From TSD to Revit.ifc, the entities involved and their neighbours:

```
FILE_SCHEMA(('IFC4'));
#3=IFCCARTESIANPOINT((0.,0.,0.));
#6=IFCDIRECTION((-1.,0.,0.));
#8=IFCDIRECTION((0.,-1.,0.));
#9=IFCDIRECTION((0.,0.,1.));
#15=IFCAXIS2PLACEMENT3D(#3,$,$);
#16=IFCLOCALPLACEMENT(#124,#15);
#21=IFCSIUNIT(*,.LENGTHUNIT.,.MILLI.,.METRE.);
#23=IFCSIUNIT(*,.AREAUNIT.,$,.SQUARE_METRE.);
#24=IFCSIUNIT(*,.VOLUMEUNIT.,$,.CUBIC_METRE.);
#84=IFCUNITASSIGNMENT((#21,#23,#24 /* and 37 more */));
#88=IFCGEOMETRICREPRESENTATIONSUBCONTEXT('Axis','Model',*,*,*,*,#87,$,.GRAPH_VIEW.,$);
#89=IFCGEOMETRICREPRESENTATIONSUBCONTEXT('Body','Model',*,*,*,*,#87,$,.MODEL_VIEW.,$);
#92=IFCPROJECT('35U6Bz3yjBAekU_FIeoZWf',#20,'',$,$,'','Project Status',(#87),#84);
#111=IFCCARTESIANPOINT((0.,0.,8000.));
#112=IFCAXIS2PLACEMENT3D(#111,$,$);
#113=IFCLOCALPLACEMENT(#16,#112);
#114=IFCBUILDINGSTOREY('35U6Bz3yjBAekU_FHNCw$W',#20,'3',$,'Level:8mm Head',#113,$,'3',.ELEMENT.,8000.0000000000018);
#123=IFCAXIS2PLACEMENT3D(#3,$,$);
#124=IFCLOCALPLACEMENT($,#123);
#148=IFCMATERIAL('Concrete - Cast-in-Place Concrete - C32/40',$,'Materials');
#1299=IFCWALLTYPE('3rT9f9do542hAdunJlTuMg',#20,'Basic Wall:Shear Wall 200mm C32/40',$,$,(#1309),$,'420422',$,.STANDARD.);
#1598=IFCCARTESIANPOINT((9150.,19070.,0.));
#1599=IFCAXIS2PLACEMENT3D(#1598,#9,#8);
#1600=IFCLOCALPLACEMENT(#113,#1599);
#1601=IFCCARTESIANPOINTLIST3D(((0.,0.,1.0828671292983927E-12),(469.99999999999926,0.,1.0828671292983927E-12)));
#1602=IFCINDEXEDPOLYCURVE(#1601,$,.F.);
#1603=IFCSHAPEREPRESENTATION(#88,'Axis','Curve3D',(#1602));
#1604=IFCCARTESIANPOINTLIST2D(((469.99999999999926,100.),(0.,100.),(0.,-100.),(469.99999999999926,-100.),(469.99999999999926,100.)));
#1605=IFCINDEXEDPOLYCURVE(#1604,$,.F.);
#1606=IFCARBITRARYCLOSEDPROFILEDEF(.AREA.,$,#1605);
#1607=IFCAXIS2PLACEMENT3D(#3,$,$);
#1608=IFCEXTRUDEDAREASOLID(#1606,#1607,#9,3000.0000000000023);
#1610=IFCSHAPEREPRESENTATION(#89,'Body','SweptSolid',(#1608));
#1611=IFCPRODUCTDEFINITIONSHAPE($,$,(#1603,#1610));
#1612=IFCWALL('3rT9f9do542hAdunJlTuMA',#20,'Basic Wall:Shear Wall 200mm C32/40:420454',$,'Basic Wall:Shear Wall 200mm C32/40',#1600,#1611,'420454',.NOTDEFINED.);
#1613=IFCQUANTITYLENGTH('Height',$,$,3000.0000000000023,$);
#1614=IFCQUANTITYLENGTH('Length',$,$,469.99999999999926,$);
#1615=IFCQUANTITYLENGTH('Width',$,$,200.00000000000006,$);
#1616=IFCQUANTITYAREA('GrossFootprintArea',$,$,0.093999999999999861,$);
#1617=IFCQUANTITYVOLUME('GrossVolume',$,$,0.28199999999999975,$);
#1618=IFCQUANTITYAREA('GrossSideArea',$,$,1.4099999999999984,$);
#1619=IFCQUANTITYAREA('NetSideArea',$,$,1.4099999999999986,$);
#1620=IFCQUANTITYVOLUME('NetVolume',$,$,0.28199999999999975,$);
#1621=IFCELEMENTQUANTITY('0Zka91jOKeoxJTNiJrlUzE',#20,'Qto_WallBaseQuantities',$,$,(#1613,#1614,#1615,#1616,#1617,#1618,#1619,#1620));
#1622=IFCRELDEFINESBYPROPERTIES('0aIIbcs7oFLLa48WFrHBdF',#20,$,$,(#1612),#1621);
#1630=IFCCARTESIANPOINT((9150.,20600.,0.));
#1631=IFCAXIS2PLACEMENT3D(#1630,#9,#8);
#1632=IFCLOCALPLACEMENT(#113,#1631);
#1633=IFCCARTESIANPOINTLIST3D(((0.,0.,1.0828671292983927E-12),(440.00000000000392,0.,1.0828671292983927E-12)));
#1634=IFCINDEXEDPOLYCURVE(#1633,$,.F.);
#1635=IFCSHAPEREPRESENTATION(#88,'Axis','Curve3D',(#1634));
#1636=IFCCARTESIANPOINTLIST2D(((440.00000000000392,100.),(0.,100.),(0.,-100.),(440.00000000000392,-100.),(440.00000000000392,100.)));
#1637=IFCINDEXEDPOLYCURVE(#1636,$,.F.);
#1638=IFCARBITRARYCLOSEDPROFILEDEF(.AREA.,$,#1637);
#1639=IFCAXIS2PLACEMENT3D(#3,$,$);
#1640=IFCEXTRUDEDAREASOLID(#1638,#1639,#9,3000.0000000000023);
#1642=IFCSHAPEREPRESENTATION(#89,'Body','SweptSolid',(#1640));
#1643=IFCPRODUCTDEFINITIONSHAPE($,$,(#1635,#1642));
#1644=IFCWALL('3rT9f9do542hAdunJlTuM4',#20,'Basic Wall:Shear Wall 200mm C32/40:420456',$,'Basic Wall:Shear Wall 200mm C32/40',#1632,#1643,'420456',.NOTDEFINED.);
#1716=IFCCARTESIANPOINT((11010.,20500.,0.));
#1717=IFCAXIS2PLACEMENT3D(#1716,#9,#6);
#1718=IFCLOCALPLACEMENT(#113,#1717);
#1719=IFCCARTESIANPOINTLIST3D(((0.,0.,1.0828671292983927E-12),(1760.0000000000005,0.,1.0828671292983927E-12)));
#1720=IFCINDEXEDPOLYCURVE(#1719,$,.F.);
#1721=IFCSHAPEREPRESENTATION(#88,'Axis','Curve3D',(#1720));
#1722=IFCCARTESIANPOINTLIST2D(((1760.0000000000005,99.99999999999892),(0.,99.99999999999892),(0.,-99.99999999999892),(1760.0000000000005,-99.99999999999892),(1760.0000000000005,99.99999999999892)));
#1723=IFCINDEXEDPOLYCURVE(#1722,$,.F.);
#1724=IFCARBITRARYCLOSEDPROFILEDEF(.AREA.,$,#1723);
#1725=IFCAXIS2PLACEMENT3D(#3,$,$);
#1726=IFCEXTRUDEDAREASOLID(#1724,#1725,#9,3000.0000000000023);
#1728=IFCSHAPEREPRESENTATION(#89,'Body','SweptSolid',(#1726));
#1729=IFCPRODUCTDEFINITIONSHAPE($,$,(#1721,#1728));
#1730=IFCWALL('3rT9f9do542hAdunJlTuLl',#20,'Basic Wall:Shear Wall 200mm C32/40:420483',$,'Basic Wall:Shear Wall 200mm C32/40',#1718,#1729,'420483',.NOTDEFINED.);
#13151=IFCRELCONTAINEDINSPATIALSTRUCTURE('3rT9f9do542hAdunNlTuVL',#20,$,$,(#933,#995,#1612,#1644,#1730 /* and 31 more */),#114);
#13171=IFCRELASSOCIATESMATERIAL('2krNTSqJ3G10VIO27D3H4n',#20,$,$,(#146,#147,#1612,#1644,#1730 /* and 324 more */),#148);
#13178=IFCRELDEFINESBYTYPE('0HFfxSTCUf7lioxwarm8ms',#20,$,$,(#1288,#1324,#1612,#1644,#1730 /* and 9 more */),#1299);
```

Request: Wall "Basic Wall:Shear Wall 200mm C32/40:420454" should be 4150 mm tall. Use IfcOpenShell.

```python
import ifcopenshell
import ifcopenshell.api.pset
import ifcopenshell.geom
import ifcopenshell.util.element
import ifcopenshell.util.representation
import ifcopenshell.util.shape
import ifcopenshell.util.unit

model = ifcopenshell.open("TSD to Revit.ifc")
unit_scale = ifcopenshell.util.unit.calculate_unit_scale(model)
area_scale = ifcopenshell.util.unit.calculate_unit_scale(model, "AREAUNIT")
volume_scale = ifcopenshell.util.unit.calculate_unit_scale(model, "VOLUMEUNIT")
settings = ifcopenshell.geom.settings()


def volume(element):
    """Net volume in cubic metres, openings subtracted."""
    shape = ifcopenshell.geom.create_shape(settings, element)
    return ifcopenshell.util.shape.get_volume(shape.geometry)


wall = model.by_guid("3rT9f9do542hAdunJlTuMA")
before = volume(wall)

body = ifcopenshell.util.representation.get_representation(wall, "Model", "Body")
solid = body.Items[0]
old_height = solid.Depth
solid.Depth = 4.15 / unit_scale
after = volume(wall)
thickness = 0.2  # wall thickness in metres

# Update the stored height, areas and volumes.
qto = model.by_id(ifcopenshell.util.element.get_pset(wall, "Qto_WallBaseQuantities", should_inherit=False)["id"])
ifcopenshell.api.pset.edit_qto(model, qto=qto, properties={
    "Height": solid.Depth,
    "GrossVolume": ifcopenshell.util.element.get_pset(wall, "Qto_WallBaseQuantities", "GrossVolume") * solid.Depth / old_height,
    "GrossSideArea": ifcopenshell.util.element.get_pset(wall, "Qto_WallBaseQuantities", "GrossSideArea") * solid.Depth / old_height,
    "NetSideArea": after / thickness / area_scale,
    "NetVolume": after / volume_scale,
})

print(f"height {old_height:g} -> {solid.Depth:g}, volume {before:.3f} -> {after:.3f} m3")

model.write("TSD to Revit_rev.ifc")
```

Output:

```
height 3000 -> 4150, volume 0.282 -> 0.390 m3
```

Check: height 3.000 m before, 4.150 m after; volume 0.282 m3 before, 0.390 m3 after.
